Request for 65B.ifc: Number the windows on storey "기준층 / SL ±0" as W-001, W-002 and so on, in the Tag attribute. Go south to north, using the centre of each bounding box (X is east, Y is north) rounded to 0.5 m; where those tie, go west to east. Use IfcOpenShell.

First a look at what the model holds.

```python
import ifcopenshell
import ifcopenshell.util.element
import ifcopenshell.util.placement

model = ifcopenshell.open("65B.ifc")
print(model.schema)
storey = next(s for s in model.by_type("IfcBuildingStorey") if s.Name == "기준층 / SL ±0")
windows = [e for e in ifcopenshell.util.element.get_decomposition(storey) if e.is_a("IfcWindow")]
for e in sorted(windows, key=lambda e: e.id()):
    origin = ifcopenshell.util.placement.get_local_placement(e.ObjectPlacement)[:3, 3]
    print(e.id(), e.Tag, e.Name, origin.round(2) + 0.0, sep=" | ")
```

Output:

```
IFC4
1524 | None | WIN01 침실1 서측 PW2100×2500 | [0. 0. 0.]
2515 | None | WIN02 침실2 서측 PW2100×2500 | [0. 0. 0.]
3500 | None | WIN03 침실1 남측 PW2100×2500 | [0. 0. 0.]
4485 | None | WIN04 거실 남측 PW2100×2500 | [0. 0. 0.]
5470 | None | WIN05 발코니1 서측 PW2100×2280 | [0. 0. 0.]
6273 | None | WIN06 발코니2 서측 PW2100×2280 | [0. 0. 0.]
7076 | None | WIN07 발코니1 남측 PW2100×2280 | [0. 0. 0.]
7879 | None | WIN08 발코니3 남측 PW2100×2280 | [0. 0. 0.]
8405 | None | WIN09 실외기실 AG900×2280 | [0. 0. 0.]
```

```python
import ifcopenshell
import ifcopenshell.geom
import ifcopenshell.util.element
import ifcopenshell.util.shape

model = ifcopenshell.open("65B.ifc")
settings = ifcopenshell.geom.settings()
settings.set("use-world-coords", True)


def centre(element):
    shape = ifcopenshell.geom.create_shape(settings, element)
    return ifcopenshell.util.shape.get_bbox_centroid(shape.geometry)


storey = next(s for s in model.by_type("IfcBuildingStorey") if s.Name == "기준층 / SL ±0")
windows = [e for e in ifcopenshell.util.element.get_decomposition(storey) if e.is_a("IfcWindow")]

# Insertion points can sit at a corner or the storey origin, so sort by the geometry (in metres).
centres = {e: centre(e) for e in windows}
windows.sort(key=lambda e: (round(centres[e][1] / 0.5), centres[e][0]))

for i, e in enumerate(windows, start=1):
    number = f"W-0{i:02d}"
    e.Tag = number
    print(e.id(), number)

model.write("65B_edited.ifc")
```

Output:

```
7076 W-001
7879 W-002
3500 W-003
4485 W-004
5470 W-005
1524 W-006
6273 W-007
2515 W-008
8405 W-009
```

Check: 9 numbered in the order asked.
